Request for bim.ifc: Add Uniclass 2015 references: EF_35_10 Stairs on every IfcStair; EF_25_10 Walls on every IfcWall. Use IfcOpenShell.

First a look at what the model holds.

```python
import ifcopenshell

model = ifcopenshell.open("bim.ifc")
print(model.schema)
print("classifications:", [c.Name for c in model.by_type("IfcClassification")])
for ifc_class in ("IfcDoor", "IfcRoof", "IfcStair", "IfcWall", "IfcWindow"):
    print(ifc_class, len(model.by_type(ifc_class)))
```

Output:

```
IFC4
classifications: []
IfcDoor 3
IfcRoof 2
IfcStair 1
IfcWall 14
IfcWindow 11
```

```python
import ifcopenshell
import ifcopenshell.api.classification

model = ifcopenshell.open("bim.ifc")

system = ifcopenshell.api.classification.add_classification(model, classification="Uniclass 2015")

codes = {
    "IfcStair": ("EF_35_10", "Stairs"),
    "IfcWall": ("EF_25_10", "Walls"),
}
for ifc_class, (code, name) in codes.items():
    products = model.by_type(ifc_class)
    ifcopenshell.api.classification.add_reference(
        model, products=products, classification=system, identification=code, name=name
    )
    print(code, len(products))

model.write("bim_rev.ifc")
```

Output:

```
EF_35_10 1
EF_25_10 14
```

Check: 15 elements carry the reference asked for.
